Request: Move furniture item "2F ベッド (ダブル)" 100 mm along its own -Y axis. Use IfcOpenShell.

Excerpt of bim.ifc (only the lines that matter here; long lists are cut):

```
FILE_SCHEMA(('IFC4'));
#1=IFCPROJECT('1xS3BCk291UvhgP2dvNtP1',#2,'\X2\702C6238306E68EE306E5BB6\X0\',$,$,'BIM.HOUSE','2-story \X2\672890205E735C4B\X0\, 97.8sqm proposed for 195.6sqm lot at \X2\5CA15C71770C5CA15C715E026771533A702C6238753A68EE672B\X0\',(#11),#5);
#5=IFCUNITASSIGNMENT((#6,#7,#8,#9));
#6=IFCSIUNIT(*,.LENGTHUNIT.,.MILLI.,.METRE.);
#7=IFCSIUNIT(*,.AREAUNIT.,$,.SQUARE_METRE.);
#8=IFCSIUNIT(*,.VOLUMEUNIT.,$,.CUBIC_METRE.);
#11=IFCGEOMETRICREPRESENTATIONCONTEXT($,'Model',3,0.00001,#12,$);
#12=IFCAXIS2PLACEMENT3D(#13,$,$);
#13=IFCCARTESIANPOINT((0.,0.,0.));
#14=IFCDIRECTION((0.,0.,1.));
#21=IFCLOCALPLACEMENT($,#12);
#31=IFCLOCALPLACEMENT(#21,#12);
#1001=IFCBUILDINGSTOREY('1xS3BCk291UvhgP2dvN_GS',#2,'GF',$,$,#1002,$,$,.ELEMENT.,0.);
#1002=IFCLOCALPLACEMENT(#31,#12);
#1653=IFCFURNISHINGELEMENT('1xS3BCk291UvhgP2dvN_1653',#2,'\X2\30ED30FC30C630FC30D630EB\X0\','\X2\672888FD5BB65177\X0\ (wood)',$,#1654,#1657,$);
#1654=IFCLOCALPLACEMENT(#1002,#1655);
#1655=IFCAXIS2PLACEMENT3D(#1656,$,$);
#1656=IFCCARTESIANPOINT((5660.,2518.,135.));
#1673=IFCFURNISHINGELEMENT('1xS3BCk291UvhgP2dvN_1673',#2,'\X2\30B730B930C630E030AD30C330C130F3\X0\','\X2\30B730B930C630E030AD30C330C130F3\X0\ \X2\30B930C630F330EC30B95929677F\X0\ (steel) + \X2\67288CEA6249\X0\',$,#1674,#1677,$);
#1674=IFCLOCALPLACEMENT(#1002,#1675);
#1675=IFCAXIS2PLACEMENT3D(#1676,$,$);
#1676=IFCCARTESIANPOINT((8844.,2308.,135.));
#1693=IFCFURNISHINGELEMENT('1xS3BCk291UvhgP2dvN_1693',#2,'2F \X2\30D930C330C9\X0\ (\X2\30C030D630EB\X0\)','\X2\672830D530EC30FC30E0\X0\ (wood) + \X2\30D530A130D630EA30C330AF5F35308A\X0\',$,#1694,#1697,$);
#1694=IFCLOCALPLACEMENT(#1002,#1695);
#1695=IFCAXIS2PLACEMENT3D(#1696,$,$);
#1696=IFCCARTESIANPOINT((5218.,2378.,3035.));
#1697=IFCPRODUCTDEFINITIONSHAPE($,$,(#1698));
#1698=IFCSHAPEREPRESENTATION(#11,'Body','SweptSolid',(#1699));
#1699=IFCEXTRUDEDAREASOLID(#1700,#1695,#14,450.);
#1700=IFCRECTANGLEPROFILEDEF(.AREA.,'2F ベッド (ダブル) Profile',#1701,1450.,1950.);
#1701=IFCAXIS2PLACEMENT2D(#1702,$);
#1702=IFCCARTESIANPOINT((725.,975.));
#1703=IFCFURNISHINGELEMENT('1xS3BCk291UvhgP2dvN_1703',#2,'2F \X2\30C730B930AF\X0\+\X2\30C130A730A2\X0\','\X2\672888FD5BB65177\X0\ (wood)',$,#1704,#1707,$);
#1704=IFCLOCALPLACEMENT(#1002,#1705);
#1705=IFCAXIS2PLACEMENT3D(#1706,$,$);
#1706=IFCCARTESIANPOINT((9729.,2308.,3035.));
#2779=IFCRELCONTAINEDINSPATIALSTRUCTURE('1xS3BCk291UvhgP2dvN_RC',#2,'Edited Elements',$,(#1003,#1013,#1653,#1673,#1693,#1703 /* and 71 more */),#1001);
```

```python
import ifcopenshell
import ifcopenshell.api.geometry
import ifcopenshell.util.placement
import ifcopenshell.util.unit

model = ifcopenshell.open("bim.ifc")
unit_scale = ifcopenshell.util.unit.calculate_unit_scale(model)

item = model.by_guid("1xS3BCk291UvhgP2dvN_1693")
matrix = ifcopenshell.util.placement.get_local_placement(item.ObjectPlacement)
matrix[:3, 3] -= matrix[:3, 1] * 0.1 / unit_scale
ifcopenshell.api.geometry.edit_object_placement(model, product=item, matrix=matrix, is_si=False)

print(ifcopenshell.util.placement.get_local_placement(item.ObjectPlacement).round(3) + 0.0)

model.write("bim-out.ifc")
```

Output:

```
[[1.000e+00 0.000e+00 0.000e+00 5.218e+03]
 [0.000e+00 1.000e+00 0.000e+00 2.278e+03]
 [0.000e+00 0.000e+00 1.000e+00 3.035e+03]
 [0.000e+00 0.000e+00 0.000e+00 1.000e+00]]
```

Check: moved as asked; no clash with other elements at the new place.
